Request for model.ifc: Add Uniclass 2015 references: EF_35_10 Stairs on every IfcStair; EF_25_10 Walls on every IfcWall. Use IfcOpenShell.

First a look at what the model holds.

```python
import ifcopenshell

model = ifcopenshell.open("model.ifc")
print(model.schema)
print("classifications:", [c.Name for c in model.by_type("IfcClassification")])
for ifc_class in ("IfcDoor", "IfcRoof", "IfcStair", "IfcWall", "IfcWindow"):
    print(ifc_class, len(model.by_type(ifc_class)))
```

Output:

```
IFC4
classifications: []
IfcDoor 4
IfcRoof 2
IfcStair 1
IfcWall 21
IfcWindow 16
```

```python
import ifcopenshell
import ifcopenshell.api.classification

model = ifcopenshell.open("model.ifc")

system = ifcopenshell.api.classification.add_classification(model, classification="Uniclass 2015")

codes = {
    "IfcStair": ("EF_35_10", "Stairs"),
    "IfcWall": ("EF_25_10", "Walls"),
}
for ifc_class, (code, name) in codes.items():
    products = model.by_type(ifc_class)
    ifcopenshell.api.classification.add_reference(
        model, products=products, classification=system, identification=code, name=name
    )
    print(code, len(products))

model.write("model_rev.ifc")
```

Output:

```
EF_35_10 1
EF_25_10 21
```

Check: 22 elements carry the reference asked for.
